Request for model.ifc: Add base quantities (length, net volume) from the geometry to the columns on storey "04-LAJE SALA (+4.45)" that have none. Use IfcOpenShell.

First a look at what the model holds.

```python
import ifcopenshell
import ifcopenshell.util.element
import ifcopenshell.util.unit

model = ifcopenshell.open("model.ifc")
print(model.schema)
for unit_type in ("LENGTHUNIT", "AREAUNIT", "VOLUMEUNIT"):
    print(unit_type, ifcopenshell.util.unit.calculate_unit_scale(model, unit_type))
storey = next(s for s in model.by_type("IfcBuildingStorey") if s.Name == "04-LAJE SALA (+4.45)")
columns = [e for e in ifcopenshell.util.element.get_decomposition(storey) if e.is_a("IfcColumn")]
for e in sorted(columns, key=lambda e: e.id()):
    print(e.id(), e.is_a(), e.Name, list(ifcopenshell.util.element.get_psets(e, qtos_only=True)), sep=" | ")
```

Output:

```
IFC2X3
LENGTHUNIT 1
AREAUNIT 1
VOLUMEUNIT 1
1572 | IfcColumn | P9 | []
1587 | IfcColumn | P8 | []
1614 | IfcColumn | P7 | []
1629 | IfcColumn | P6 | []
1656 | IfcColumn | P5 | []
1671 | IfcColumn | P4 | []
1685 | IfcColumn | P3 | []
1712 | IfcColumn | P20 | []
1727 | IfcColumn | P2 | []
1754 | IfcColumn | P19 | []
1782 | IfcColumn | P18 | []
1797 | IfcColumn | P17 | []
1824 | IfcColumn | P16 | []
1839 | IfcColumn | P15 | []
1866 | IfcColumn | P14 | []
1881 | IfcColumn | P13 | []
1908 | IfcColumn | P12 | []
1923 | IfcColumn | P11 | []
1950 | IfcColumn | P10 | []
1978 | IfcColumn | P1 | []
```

```python
import ifcopenshell
import ifcopenshell.api.pset
import ifcopenshell.geom
import ifcopenshell.util.element
import ifcopenshell.util.shape
import ifcopenshell.util.unit

model = ifcopenshell.open("model.ifc")
unit_scale = ifcopenshell.util.unit.calculate_unit_scale(model)
volume_scale = ifcopenshell.util.unit.calculate_unit_scale(model, "VOLUMEUNIT")
settings = ifcopenshell.geom.settings()

storey = next(s for s in model.by_type("IfcBuildingStorey") if s.Name == "04-LAJE SALA (+4.45)")
columns = [e for e in ifcopenshell.util.element.get_decomposition(storey) if e.is_a("IfcColumn")]

for e in sorted(columns, key=lambda e: e.id()):
    if ifcopenshell.util.element.get_psets(e, qtos_only=True, should_inherit=False):
        continue
    # Geometry comes back in metres, in the element's own axes.
    shape = ifcopenshell.geom.create_shape(settings, e)
    values = {
        "Length": ifcopenshell.util.shape.get_z(shape.geometry) / unit_scale,
        "NetVolume": ifcopenshell.util.shape.get_volume(shape.geometry) / volume_scale,
    }
    qto = ifcopenshell.api.pset.add_qto(model, product=e, name="BaseQuantities")
    ifcopenshell.api.pset.edit_qto(model, qto=qto, properties=values)
    print(e.id(), {k: round(v, 3) for k, v in values.items()})

model.write("model_updated.ifc")
```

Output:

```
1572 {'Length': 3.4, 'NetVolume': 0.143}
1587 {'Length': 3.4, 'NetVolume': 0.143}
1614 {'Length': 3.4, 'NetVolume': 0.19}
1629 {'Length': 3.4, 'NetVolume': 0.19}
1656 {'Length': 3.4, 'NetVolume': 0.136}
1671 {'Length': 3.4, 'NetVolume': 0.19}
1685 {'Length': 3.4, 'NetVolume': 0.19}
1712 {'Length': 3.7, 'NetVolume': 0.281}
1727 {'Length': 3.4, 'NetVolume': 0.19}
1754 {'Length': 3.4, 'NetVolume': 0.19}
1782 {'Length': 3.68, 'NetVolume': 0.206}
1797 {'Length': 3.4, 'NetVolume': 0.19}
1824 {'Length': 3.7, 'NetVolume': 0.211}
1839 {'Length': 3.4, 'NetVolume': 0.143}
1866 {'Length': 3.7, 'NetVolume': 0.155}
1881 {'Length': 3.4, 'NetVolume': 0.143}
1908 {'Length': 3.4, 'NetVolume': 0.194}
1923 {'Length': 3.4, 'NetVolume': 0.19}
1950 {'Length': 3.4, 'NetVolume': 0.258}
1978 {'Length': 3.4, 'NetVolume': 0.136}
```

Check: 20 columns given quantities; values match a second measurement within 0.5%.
